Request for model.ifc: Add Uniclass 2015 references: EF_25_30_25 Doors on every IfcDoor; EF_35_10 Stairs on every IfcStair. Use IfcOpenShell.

First a look at what the model holds.

```python
import ifcopenshell

model = ifcopenshell.open("model.ifc")
print(model.schema)
print("classifications:", [c.Name for c in model.by_type("IfcClassification")])
for ifc_class in ("IfcDoor", "IfcRoof", "IfcStair", "IfcWall", "IfcWindow"):
    print(ifc_class, len(model.by_type(ifc_class)))
```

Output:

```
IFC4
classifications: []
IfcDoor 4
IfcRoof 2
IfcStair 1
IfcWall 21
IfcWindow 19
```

```python
import ifcopenshell
import ifcopenshell.api.classification

model = ifcopenshell.open("model.ifc")

system = ifcopenshell.api.classification.add_classification(model, classification="Uniclass 2015")

codes = {
    "IfcDoor": ("EF_25_30_25", "Doors"),
    "IfcStair": ("EF_35_10", "Stairs"),
}
for ifc_class, (code, name) in codes.items():
    products = model.by_type(ifc_class)
    ifcopenshell.api.classification.add_reference(
        model, products=products, classification=system, identification=code, name=name
    )
    print(code, len(products))

model.write("model-out.ifc")
```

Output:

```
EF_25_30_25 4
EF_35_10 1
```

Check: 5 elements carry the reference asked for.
